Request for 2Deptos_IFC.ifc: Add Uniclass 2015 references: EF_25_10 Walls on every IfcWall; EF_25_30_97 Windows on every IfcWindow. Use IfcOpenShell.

First a look at what the model holds.

```python
import ifcopenshell

model = ifcopenshell.open("2Deptos_IFC.ifc")
print(model.schema)
print("classifications:", [c.Name for c in model.by_type("IfcClassification")])
for ifc_class in ("IfcDoor", "IfcRoof", "IfcStair", "IfcWall", "IfcWindow"):
    print(ifc_class, len(model.by_type(ifc_class)))
```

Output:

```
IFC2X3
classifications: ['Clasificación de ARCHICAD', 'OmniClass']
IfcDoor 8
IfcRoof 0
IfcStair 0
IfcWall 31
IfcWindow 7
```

```python
import ifcopenshell
import ifcopenshell.api.classification

model = ifcopenshell.open("2Deptos_IFC.ifc")

# IFC2X3 requires Source and Edition and has no link from the project to the system.
system = model.create_entity("IfcClassification", Source="NBS", Edition="2015", Name="Uniclass 2015")

codes = {
    "IfcWall": ("EF_25_10", "Walls"),
    "IfcWindow": ("EF_25_30_97", "Windows"),
}
for ifc_class, (code, name) in codes.items():
    products = model.by_type(ifc_class)
    ifcopenshell.api.classification.add_reference(
        model, products=products, classification=system, identification=code, name=name
    )
    print(code, len(products))

model.write("2Deptos_IFC-out.ifc")
```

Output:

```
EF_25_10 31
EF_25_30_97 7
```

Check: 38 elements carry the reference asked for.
